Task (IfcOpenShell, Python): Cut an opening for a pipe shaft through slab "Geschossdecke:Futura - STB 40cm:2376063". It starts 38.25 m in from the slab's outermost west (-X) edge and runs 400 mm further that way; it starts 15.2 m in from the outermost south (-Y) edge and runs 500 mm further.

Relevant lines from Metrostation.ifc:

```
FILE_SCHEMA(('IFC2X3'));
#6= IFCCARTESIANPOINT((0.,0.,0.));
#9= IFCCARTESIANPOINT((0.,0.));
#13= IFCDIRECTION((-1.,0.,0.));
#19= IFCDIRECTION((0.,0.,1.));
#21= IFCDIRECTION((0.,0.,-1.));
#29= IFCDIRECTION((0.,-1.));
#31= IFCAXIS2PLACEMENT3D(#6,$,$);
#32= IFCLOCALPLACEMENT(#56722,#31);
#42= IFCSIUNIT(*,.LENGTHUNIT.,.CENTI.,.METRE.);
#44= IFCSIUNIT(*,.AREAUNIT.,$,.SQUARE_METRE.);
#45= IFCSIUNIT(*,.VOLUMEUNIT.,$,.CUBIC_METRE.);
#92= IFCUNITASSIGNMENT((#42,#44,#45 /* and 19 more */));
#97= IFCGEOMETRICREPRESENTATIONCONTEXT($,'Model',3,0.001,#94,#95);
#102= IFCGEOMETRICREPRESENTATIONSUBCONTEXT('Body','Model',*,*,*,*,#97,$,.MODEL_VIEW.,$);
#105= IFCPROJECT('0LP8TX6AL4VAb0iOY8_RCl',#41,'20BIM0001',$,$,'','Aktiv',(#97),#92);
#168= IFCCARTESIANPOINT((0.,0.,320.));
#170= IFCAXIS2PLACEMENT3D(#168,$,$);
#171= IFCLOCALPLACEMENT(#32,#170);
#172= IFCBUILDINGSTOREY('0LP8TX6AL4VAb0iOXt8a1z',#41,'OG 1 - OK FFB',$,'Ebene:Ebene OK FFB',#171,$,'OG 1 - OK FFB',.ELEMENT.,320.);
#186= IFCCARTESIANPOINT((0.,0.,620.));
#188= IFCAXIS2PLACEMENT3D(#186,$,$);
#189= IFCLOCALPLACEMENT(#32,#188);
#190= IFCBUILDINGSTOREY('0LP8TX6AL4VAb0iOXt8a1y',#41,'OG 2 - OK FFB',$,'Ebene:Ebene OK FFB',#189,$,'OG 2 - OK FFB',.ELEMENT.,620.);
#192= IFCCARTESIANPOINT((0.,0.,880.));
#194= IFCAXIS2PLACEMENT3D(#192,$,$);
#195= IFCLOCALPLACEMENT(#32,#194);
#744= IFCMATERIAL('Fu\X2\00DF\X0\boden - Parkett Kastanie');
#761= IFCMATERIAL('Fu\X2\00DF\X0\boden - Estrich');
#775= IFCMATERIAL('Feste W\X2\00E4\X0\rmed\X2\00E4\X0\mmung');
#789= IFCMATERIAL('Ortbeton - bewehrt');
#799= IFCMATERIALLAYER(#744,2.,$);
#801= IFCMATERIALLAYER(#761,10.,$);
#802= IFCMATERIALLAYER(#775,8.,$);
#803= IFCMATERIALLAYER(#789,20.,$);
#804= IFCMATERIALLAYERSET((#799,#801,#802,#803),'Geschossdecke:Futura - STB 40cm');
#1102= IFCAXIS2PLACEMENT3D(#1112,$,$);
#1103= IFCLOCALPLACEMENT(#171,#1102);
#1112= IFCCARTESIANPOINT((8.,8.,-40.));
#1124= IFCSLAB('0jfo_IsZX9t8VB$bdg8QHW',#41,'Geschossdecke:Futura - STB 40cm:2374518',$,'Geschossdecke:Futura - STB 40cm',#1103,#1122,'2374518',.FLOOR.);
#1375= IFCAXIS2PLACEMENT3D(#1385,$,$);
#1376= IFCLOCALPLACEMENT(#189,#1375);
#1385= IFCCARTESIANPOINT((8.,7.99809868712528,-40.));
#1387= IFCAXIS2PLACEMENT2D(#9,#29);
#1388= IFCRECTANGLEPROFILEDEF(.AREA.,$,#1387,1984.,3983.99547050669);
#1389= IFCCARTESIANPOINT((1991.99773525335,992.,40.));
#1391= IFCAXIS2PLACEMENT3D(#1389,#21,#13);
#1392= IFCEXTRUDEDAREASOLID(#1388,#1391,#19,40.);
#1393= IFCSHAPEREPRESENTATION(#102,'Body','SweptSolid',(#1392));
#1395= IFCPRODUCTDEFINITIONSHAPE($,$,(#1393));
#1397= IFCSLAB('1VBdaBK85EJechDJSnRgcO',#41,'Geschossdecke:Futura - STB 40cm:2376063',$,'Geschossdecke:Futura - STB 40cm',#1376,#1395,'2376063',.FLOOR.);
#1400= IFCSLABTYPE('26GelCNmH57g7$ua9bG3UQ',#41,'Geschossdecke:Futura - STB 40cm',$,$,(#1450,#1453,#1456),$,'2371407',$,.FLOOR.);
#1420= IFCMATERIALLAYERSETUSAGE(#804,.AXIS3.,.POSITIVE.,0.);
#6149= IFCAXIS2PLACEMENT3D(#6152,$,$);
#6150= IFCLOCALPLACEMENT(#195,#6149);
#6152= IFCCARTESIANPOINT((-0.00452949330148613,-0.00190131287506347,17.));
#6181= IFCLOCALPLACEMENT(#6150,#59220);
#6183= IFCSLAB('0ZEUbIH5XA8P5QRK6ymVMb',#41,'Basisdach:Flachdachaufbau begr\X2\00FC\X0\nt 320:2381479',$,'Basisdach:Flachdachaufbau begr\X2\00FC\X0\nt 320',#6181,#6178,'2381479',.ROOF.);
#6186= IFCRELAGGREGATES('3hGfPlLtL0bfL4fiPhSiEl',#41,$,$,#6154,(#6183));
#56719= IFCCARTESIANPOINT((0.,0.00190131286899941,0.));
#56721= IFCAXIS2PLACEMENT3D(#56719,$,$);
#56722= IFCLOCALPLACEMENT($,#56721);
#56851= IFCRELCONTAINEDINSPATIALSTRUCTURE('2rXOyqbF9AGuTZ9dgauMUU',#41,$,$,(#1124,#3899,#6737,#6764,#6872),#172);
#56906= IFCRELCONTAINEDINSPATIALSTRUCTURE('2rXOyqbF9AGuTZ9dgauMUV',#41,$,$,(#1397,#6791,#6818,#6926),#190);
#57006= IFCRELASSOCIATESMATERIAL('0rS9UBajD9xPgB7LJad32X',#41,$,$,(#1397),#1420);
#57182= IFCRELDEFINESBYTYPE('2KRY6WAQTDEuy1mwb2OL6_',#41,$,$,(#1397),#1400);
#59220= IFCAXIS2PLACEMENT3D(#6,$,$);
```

```python
import numpy as np
import ifcopenshell
import ifcopenshell.api.feature
import ifcopenshell.api.geometry
import ifcopenshell.api.root
import ifcopenshell.geom
import ifcopenshell.util.placement
import ifcopenshell.util.representation
import ifcopenshell.util.shape
import ifcopenshell.util.unit

model = ifcopenshell.open("Metrostation.ifc")
unit_scale = ifcopenshell.util.unit.calculate_unit_scale(model)
settings = ifcopenshell.geom.settings()


def volume(element):
    """Net volume in cubic metres, openings subtracted."""
    shape = ifcopenshell.geom.create_shape(settings, element)
    return ifcopenshell.util.shape.get_volume(shape.geometry)


slab = model.by_id(1397)
before = volume(slab)

# Extent in the slab's own axes, in metres. The edges named are its -X and -Y sides.
slab_shape = ifcopenshell.geom.create_shape(settings, slab)
vertices = ifcopenshell.util.shape.get_vertices(slab_shape.geometry)
x_min, y_min, bottom = vertices.min(axis=0)
top = vertices[:, 2].max()

opening = ifcopenshell.api.root.create_entity(model, ifc_class="IfcOpeningElement", name="Pipe shaft opening")
context = ifcopenshell.util.representation.get_context(model, "Model", "Body", "MODEL_VIEW")
width, depth = 0.4, 0.5
outline = [(0.0, 0.0), (width, 0.0), (width, depth), (0.0, depth), (0.0, 0.0)]
# Overshoot both faces by 50 mm so the cut is clean.
shape = ifcopenshell.api.geometry.add_slab_representation(
    model, context=context, depth=top - bottom + 0.1, polyline=outline
)
ifcopenshell.api.geometry.assign_representation(model, product=opening, representation=shape)

matrix = ifcopenshell.util.placement.get_local_placement(slab.ObjectPlacement)
matrix[:, 3] = matrix @ np.append(np.array([x_min + 38.25, y_min + 15.2, bottom - 0.05]) / unit_scale, 1.0)
ifcopenshell.api.geometry.edit_object_placement(model, product=opening, matrix=matrix, is_si=False)
ifcopenshell.api.feature.add_feature(model, feature=opening, element=slab)

after = volume(slab)

print(f"slab volume {before:.3f} -> {after:.3f} m3")

model.write("Metrostation-out.ifc")
```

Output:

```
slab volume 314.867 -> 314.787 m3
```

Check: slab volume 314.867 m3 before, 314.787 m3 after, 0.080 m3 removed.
